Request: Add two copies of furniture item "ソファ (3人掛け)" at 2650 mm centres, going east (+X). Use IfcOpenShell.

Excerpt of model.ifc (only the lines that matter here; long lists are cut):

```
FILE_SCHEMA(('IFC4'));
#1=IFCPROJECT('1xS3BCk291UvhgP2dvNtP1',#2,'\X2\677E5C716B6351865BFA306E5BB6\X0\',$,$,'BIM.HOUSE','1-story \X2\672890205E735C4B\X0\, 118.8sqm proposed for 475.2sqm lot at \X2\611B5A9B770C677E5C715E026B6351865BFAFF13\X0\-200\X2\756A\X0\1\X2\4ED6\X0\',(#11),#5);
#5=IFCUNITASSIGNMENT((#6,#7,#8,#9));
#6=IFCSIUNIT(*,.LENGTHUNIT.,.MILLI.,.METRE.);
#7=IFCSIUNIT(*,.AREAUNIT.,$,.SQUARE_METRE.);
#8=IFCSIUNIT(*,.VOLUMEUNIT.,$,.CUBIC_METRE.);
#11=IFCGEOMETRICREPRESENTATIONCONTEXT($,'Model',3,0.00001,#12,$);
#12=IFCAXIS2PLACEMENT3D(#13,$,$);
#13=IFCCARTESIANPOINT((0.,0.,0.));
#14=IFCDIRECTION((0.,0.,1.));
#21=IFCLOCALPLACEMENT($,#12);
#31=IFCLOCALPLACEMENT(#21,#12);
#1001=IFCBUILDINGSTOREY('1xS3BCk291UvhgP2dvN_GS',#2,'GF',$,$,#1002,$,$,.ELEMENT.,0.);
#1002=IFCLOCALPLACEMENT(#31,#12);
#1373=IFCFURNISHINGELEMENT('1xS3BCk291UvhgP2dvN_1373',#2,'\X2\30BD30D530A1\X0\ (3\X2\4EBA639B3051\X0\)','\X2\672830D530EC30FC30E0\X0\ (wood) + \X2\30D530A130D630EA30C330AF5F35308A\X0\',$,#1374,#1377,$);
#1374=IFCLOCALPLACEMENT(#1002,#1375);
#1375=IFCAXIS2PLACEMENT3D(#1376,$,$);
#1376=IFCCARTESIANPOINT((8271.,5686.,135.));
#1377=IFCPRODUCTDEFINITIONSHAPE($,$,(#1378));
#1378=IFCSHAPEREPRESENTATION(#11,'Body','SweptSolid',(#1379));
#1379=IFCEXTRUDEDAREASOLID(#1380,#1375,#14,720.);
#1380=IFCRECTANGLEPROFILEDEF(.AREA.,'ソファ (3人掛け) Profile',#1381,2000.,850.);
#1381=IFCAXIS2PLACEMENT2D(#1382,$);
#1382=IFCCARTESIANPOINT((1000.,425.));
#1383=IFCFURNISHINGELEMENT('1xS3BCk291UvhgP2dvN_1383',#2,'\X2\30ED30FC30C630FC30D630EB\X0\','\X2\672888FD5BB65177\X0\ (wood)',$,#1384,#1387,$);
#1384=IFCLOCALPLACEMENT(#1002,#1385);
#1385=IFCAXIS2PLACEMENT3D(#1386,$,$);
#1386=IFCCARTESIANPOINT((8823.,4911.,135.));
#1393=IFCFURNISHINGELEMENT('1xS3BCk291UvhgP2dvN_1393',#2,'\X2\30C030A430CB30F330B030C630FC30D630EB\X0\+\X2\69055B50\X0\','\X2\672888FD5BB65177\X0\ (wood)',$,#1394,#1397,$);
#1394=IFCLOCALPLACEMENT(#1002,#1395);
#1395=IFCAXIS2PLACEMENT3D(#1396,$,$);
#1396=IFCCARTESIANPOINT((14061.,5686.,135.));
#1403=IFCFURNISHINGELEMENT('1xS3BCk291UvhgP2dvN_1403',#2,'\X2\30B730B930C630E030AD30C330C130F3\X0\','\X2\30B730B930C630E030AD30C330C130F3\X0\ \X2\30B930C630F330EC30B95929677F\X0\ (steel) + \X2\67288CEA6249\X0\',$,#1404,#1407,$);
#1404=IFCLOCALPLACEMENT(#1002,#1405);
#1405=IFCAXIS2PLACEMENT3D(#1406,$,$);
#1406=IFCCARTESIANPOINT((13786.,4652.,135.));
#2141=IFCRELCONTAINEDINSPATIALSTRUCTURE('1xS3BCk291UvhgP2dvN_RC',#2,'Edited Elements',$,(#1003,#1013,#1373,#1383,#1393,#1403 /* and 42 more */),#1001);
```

```python
import numpy as np
import ifcopenshell
import ifcopenshell.api.geometry
import ifcopenshell.api.root
import ifcopenshell.util.element
import ifcopenshell.util.placement

model = ifcopenshell.open("model.ifc")


def reuse_history(source, copy):
    """copy_class also copies each property set's owner history, people and application; keep the originals."""
    for rel in copy.IsDefinedBy:
        if rel.is_a("IfcRelDefinesByProperties") and (history := rel.RelatingPropertyDefinition.OwnerHistory):
            rel.RelatingPropertyDefinition.OwnerHistory = source.OwnerHistory
            ifcopenshell.util.element.remove_deep2(model, history)


source = model.by_guid("1xS3BCk291UvhgP2dvN_1373")
base = ifcopenshell.util.placement.get_local_placement(source.ObjectPlacement)
step = np.array([1.0, 0.0, 0.0]) * 2650.0

for i in range(1, 3):
    copy = ifcopenshell.api.root.copy_class(model, product=source)
    copy.Representation = ifcopenshell.util.element.copy_deep(
        model, source.Representation, exclude=["IfcGeometricRepresentationContext", "IfcRepresentationMap"]
    )
    reuse_history(source, copy)
    matrix = base.copy()
    matrix[:3, 3] += i * step
    print("added at", matrix[:3, 3].round(3) + 0.0)
    ifcopenshell.api.geometry.edit_object_placement(model, product=copy, matrix=matrix, is_si=False)

model.write("model_v2.ifc")
```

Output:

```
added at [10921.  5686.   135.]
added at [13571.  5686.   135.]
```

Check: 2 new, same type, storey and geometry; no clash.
